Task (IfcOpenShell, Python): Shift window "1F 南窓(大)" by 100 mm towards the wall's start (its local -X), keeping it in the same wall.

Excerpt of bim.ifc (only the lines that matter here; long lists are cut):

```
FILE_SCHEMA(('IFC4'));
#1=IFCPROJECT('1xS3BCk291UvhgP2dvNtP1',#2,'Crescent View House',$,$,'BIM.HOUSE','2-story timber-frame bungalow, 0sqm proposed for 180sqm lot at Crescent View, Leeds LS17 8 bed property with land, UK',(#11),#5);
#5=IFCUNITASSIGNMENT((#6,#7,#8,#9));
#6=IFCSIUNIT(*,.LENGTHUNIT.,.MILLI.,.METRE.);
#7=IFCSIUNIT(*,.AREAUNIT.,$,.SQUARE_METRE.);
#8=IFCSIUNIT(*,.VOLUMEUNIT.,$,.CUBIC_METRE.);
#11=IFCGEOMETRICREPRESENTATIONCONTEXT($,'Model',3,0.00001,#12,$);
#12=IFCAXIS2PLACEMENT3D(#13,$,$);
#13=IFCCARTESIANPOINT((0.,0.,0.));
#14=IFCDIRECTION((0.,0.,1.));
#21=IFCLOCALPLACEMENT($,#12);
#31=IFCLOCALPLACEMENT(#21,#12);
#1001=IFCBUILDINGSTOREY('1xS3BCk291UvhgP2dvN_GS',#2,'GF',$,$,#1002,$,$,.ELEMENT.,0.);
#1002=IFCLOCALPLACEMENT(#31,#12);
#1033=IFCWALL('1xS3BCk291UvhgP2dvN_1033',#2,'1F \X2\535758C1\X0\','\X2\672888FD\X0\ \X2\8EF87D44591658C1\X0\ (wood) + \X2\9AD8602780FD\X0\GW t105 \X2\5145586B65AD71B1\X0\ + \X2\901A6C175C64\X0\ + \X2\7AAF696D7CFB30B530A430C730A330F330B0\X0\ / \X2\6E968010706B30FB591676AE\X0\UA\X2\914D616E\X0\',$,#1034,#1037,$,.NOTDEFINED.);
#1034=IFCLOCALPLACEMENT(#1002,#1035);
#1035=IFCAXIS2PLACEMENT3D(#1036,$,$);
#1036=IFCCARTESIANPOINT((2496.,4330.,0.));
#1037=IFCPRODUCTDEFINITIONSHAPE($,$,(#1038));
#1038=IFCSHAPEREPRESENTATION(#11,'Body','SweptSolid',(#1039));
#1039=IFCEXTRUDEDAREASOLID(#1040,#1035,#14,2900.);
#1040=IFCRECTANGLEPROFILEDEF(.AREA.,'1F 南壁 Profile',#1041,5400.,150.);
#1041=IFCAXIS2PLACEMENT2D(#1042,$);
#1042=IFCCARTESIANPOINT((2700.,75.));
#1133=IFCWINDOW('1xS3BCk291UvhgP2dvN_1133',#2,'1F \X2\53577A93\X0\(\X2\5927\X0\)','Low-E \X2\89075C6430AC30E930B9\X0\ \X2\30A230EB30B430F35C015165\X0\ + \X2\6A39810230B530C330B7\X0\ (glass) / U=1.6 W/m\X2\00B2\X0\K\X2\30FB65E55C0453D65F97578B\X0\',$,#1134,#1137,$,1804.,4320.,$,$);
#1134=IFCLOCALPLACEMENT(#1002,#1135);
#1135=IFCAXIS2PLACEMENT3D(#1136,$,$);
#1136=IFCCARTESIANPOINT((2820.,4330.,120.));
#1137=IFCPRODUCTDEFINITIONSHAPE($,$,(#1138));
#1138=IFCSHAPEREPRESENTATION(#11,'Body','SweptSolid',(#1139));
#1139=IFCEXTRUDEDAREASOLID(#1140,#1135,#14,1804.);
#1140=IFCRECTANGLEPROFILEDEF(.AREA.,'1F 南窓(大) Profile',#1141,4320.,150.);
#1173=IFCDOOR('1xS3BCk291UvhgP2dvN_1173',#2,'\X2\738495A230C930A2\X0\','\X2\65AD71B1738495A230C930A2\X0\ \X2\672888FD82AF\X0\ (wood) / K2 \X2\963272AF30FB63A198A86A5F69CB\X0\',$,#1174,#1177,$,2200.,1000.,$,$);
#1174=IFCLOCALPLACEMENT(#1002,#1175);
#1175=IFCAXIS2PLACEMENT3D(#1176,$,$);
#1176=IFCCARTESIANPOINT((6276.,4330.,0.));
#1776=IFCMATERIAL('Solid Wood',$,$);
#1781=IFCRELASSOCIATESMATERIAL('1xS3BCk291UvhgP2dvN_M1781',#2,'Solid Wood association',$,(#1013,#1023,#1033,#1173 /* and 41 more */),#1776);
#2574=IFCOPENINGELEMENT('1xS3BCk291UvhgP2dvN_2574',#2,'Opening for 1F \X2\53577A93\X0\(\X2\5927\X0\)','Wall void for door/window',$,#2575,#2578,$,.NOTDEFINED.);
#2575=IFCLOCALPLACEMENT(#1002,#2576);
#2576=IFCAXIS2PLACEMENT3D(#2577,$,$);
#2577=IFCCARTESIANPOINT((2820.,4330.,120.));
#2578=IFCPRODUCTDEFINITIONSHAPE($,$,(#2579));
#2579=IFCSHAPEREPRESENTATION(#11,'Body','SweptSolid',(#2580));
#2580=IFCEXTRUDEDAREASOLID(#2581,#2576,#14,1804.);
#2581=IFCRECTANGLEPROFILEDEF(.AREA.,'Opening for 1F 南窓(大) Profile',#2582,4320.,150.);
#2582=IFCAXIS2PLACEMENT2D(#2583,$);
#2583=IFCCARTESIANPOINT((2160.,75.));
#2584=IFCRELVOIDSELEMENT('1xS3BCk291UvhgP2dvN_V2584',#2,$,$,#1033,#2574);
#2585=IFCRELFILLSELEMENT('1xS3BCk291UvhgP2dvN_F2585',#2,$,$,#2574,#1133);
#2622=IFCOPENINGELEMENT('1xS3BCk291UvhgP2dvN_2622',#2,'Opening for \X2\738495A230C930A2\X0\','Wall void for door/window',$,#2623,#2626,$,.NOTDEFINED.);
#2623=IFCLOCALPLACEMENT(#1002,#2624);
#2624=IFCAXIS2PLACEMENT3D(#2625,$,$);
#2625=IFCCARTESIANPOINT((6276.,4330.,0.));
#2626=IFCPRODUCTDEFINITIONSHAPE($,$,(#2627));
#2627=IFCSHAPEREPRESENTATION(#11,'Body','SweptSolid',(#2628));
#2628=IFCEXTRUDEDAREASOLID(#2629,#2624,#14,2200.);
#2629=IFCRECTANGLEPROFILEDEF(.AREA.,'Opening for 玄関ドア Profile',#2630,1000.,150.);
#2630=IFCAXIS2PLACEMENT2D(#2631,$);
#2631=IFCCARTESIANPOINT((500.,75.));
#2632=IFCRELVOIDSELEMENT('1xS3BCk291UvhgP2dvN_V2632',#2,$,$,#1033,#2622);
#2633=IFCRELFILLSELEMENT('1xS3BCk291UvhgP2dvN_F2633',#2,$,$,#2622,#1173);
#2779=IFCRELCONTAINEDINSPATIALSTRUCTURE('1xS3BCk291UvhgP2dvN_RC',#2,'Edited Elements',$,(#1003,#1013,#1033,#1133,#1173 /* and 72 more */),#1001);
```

```python
import ifcopenshell
import ifcopenshell.api.geometry
import ifcopenshell.util.placement
import ifcopenshell.util.unit

model = ifcopenshell.open("bim.ifc")
unit_scale = ifcopenshell.util.unit.calculate_unit_scale(model)

window = model.by_guid("1xS3BCk291UvhgP2dvN_1133")
opening = window.FillsVoids[0].RelatingOpeningElement
wall = opening.VoidsElements[0].RelatingBuildingElement

wall_matrix = ifcopenshell.util.placement.get_local_placement(wall.ObjectPlacement)
shift = wall_matrix[:3, 0] * -0.1 / unit_scale
before = ifcopenshell.util.placement.get_local_placement(window.ObjectPlacement)[:3, 3].copy()

# The window is not placed relative to its opening, so move both.
for product in (opening, window):
    matrix = ifcopenshell.util.placement.get_local_placement(product.ObjectPlacement)
    matrix[:3, 3] += shift
    ifcopenshell.api.geometry.edit_object_placement(model, product=product, matrix=matrix, is_si=False)

after = ifcopenshell.util.placement.get_local_placement(window.ObjectPlacement)[:3, 3]
print("window moved by", (after - before).round(3) + 0.0)

model.write("bim_rev.ifc")
```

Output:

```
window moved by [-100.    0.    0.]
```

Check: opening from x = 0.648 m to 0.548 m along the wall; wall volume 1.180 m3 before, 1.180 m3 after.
